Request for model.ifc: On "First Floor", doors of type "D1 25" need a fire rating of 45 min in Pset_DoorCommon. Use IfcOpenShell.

First a look at what the model holds.

```python
import ifcopenshell
import ifcopenshell.util.element

model = ifcopenshell.open("model.ifc")
print(model.schema)
storey = next(s for s in model.by_type("IfcBuildingStorey") if s.Name == "First Floor")
doors = [e for e in ifcopenshell.util.element.get_decomposition(storey) if e.is_a("IfcDoor")]
seen = {}
for e in doors:
    element_type = ifcopenshell.util.element.get_type(e)
    key = (element_type.Name if element_type != e and element_type else None, ifcopenshell.util.element.get_pset(e, "Pset_DoorCommon", "FireRating"))
    seen[key] = seen.get(key, 0) + 1
for (name, value), count in sorted(seen.items(), key=str):
    print(count, "x", name, "|", value)
```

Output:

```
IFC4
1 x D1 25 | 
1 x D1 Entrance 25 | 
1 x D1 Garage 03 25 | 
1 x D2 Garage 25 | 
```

```python
import ifcopenshell
import ifcopenshell.api.pset
import ifcopenshell.util.element

model = ifcopenshell.open("model.ifc")

storey = next(s for s in model.by_type("IfcBuildingStorey") if s.Name == "First Floor")
doors = [e for e in ifcopenshell.util.element.get_decomposition(storey) if e.is_a("IfcDoor")]

count = 0
for e in doors:
    element_type = ifcopenshell.util.element.get_type(e)
    if element_type in (None, e) or element_type.Name != "D1 25":
        continue
    # add_pset returns the element's existing set when there is one.
    pset = ifcopenshell.api.pset.add_pset(model, product=e, name="Pset_DoorCommon")
    ifcopenshell.api.pset.edit_pset(model, pset=pset, properties={"FireRating": "45 min"})
    count += 1

print(count, "doors updated")

model.write("model_v2.ifc")
```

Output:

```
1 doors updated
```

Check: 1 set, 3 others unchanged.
